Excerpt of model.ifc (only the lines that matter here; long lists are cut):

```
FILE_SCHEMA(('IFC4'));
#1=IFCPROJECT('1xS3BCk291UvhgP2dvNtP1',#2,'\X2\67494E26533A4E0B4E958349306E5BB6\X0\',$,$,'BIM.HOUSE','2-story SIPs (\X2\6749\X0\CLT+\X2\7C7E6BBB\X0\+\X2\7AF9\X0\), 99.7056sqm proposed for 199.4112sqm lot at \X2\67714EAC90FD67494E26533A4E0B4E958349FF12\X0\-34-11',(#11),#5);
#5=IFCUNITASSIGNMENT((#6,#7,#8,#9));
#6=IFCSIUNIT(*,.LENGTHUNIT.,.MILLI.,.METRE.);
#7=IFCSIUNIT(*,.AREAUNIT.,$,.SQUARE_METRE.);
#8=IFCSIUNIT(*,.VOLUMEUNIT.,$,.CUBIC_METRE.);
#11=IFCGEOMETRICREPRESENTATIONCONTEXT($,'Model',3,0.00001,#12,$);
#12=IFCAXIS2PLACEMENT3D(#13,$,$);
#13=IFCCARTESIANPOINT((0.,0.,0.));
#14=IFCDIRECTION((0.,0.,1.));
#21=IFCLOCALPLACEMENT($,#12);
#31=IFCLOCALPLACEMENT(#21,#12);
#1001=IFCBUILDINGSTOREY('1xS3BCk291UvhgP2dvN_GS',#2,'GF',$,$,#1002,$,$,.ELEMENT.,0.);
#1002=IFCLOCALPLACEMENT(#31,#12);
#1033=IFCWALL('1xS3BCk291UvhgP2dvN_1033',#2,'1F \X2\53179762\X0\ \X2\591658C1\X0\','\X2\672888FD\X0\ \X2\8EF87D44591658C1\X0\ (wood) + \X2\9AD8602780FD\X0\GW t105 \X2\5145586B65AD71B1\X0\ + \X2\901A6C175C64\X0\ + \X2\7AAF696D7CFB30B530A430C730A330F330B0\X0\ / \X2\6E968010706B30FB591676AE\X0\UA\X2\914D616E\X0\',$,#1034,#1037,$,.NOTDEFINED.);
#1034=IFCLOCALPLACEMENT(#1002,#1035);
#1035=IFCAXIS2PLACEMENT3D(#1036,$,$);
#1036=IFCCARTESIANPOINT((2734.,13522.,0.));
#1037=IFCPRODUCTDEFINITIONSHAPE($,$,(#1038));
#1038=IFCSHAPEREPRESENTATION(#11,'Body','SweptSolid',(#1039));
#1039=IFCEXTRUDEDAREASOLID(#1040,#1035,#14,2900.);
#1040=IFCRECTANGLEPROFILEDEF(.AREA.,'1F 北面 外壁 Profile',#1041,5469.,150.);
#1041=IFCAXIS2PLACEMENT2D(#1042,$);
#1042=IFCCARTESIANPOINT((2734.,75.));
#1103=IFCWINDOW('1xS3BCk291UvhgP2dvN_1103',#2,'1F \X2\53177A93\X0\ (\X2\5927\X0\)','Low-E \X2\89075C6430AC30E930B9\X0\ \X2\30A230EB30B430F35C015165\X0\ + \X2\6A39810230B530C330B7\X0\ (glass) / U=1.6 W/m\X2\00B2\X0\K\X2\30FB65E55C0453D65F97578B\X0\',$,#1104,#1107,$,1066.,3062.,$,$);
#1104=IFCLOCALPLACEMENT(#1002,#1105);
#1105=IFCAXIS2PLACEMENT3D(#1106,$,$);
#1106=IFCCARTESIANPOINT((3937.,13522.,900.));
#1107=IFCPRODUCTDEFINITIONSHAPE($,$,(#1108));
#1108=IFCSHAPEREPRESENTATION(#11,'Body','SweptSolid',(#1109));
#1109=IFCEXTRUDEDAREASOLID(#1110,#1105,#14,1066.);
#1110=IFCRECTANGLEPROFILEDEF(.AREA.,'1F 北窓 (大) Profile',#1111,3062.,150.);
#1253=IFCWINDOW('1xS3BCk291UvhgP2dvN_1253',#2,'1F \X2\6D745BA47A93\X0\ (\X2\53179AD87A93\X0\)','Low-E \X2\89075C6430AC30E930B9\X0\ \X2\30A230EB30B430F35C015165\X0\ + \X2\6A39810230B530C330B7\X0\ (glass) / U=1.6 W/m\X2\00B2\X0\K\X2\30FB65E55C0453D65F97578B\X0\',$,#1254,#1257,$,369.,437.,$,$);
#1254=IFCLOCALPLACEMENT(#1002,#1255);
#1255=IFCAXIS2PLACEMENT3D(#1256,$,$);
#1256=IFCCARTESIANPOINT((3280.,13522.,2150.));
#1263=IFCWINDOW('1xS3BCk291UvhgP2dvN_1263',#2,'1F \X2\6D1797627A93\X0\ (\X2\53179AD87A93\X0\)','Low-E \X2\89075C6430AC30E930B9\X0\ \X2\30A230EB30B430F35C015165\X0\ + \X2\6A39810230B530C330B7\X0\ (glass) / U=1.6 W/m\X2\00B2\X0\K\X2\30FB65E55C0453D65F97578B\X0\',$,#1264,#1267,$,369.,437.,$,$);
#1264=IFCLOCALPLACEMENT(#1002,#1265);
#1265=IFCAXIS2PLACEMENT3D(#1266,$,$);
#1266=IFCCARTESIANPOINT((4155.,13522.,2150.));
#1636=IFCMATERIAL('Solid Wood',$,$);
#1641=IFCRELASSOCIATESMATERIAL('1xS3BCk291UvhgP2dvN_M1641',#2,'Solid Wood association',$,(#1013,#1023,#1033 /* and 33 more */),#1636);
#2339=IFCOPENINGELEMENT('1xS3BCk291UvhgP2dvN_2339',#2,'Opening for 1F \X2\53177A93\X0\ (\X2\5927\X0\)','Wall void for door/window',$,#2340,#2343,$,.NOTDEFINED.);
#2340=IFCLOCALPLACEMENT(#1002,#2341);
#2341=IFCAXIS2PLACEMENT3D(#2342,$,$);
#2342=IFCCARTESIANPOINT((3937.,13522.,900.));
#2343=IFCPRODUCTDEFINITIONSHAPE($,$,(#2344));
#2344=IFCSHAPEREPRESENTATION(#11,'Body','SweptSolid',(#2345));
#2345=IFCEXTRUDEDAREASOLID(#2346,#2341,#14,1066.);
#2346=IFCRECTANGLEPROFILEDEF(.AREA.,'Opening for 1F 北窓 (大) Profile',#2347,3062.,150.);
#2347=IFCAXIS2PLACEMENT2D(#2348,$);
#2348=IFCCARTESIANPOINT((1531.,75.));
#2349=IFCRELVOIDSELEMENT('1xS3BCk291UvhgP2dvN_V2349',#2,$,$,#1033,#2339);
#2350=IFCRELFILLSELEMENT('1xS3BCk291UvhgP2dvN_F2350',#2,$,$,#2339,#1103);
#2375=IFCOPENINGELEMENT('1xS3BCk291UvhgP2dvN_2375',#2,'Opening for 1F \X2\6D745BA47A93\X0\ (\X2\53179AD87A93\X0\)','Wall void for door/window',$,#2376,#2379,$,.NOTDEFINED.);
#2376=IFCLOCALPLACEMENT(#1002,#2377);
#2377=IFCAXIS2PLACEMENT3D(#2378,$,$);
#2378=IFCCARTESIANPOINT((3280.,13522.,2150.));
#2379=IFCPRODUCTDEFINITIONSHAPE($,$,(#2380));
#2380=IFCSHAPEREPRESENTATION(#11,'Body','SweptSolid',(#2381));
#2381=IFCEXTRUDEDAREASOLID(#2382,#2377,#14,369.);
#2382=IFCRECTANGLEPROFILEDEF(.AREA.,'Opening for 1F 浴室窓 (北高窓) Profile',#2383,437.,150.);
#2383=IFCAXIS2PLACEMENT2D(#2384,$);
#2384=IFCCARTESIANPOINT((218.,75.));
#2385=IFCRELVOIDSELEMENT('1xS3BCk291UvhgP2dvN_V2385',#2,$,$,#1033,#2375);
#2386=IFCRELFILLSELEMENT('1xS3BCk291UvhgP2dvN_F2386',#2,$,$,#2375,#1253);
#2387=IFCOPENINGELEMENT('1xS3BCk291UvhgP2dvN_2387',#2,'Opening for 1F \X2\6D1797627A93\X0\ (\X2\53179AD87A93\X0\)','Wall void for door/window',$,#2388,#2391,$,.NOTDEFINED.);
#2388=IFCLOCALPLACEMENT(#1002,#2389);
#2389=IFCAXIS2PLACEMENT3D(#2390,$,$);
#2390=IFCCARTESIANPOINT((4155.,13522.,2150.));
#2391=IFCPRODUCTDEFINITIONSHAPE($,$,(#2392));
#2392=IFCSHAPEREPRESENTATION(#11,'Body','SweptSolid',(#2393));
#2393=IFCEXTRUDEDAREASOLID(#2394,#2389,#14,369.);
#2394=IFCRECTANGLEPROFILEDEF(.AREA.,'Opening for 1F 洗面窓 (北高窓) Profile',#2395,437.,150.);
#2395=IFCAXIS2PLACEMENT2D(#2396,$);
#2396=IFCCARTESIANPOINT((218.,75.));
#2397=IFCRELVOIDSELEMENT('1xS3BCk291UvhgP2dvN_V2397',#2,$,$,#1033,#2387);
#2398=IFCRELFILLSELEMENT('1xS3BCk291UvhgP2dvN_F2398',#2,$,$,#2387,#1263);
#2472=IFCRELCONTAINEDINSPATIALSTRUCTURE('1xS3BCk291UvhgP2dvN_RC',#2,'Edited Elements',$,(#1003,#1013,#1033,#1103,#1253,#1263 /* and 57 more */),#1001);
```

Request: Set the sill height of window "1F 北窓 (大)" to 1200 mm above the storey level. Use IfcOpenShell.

```python
import numpy as np
import ifcopenshell
import ifcopenshell.api.geometry
import ifcopenshell.geom
import ifcopenshell.util.element
import ifcopenshell.util.placement
import ifcopenshell.util.shape
import ifcopenshell.util.unit

model = ifcopenshell.open("model.ifc")
unit_scale = ifcopenshell.util.unit.calculate_unit_scale(model)

window = model.by_guid("1xS3BCk291UvhgP2dvN_1103")
opening = window.FillsVoids[0].RelatingOpeningElement
storey = ifcopenshell.util.element.get_container(window, ifc_class="IfcBuildingStorey")
level = ifcopenshell.util.placement.get_local_placement(storey.ObjectPlacement)[2, 3]

# The opening's origin need not be at the sill, so measure its lowest point.
shape = ifcopenshell.geom.create_shape(ifcopenshell.geom.settings(), opening)
bottom = ifcopenshell.util.shape.get_shape_bottom_elevation(shape, shape.geometry) / unit_scale
dz = level + 1.2 / unit_scale - bottom

shift = np.array([0.0, 0.0, dz])
# The window is not placed relative to its opening, so move both.
for product in (opening, window):
    matrix = ifcopenshell.util.placement.get_local_placement(product.ObjectPlacement)
    matrix[:3, 3] += shift
    ifcopenshell.api.geometry.edit_object_placement(model, product=product, matrix=matrix, is_si=False)

print(f"moved by {dz * unit_scale:+.3f} m")

model.write("model_edited.ifc")
```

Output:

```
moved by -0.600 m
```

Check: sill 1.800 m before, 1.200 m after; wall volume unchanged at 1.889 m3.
